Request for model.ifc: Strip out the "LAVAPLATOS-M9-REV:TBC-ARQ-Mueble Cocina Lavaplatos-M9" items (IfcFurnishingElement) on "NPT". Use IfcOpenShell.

First a look at what the model holds.

```python
import ifcopenshell
import ifcopenshell.util.element

model = ifcopenshell.open("model.ifc")
print(model.schema)
storey = next(s for s in model.by_type("IfcBuildingStorey") if s.Name == "NPT")
furniture = [e for e in ifcopenshell.util.element.get_decomposition(storey) if e.is_a("IfcFurnishingElement")]
seen = {}
for e in furniture:
    element_type = ifcopenshell.util.element.get_type(e)
    name = element_type.Name if element_type not in (None, e) else None
    seen[name] = seen.get(name, 0) + 1
for name, count in sorted(seen.items(), key=str):
    print(count, "x", name)
```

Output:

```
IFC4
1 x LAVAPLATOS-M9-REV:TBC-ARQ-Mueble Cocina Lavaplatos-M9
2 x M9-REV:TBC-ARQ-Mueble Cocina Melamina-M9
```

```python
import ifcopenshell
import ifcopenshell.api.root
import ifcopenshell.util.element

model = ifcopenshell.open("model.ifc")

storey = next(s for s in model.by_type("IfcBuildingStorey") if s.Name == "NPT")
furniture = [e for e in ifcopenshell.util.element.get_decomposition(storey) if e.is_a("IfcFurnishingElement")]
targets = [e for e in furniture if (t := ifcopenshell.util.element.get_type(e)) not in (None, e) and t.Name == "LAVAPLATOS-M9-REV:TBC-ARQ-Mueble Cocina Lavaplatos-M9"]

for e in targets:
    ifcopenshell.api.root.remove_product(model, product=e)
print(len(targets), "removed")

model.write("model_updated.ifc")
```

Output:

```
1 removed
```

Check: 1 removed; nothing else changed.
